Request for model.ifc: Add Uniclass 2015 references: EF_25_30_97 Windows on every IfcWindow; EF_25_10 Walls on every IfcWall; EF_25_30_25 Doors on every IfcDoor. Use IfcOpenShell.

First a look at what the model holds.

```python
import ifcopenshell

model = ifcopenshell.open("model.ifc")
print(model.schema)
print("classifications:", [c.Name for c in model.by_type("IfcClassification")])
for ifc_class in ("IfcDoor", "IfcRoof", "IfcStair", "IfcWall", "IfcWindow"):
    print(ifc_class, len(model.by_type(ifc_class)))
```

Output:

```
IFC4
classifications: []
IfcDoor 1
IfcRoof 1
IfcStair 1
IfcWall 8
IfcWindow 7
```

```python
import ifcopenshell
import ifcopenshell.api.classification

model = ifcopenshell.open("model.ifc")

system = ifcopenshell.api.classification.add_classification(model, classification="Uniclass 2015")

codes = {
    "IfcWindow": ("EF_25_30_97", "Windows"),
    "IfcWall": ("EF_25_10", "Walls"),
    "IfcDoor": ("EF_25_30_25", "Doors"),
}
for ifc_class, (code, name) in codes.items():
    products = model.by_type(ifc_class)
    ifcopenshell.api.classification.add_reference(
        model, products=products, classification=system, identification=code, name=name
    )
    print(code, len(products))

model.write("model_edited.ifc")
```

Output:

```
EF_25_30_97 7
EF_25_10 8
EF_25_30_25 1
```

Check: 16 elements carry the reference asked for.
